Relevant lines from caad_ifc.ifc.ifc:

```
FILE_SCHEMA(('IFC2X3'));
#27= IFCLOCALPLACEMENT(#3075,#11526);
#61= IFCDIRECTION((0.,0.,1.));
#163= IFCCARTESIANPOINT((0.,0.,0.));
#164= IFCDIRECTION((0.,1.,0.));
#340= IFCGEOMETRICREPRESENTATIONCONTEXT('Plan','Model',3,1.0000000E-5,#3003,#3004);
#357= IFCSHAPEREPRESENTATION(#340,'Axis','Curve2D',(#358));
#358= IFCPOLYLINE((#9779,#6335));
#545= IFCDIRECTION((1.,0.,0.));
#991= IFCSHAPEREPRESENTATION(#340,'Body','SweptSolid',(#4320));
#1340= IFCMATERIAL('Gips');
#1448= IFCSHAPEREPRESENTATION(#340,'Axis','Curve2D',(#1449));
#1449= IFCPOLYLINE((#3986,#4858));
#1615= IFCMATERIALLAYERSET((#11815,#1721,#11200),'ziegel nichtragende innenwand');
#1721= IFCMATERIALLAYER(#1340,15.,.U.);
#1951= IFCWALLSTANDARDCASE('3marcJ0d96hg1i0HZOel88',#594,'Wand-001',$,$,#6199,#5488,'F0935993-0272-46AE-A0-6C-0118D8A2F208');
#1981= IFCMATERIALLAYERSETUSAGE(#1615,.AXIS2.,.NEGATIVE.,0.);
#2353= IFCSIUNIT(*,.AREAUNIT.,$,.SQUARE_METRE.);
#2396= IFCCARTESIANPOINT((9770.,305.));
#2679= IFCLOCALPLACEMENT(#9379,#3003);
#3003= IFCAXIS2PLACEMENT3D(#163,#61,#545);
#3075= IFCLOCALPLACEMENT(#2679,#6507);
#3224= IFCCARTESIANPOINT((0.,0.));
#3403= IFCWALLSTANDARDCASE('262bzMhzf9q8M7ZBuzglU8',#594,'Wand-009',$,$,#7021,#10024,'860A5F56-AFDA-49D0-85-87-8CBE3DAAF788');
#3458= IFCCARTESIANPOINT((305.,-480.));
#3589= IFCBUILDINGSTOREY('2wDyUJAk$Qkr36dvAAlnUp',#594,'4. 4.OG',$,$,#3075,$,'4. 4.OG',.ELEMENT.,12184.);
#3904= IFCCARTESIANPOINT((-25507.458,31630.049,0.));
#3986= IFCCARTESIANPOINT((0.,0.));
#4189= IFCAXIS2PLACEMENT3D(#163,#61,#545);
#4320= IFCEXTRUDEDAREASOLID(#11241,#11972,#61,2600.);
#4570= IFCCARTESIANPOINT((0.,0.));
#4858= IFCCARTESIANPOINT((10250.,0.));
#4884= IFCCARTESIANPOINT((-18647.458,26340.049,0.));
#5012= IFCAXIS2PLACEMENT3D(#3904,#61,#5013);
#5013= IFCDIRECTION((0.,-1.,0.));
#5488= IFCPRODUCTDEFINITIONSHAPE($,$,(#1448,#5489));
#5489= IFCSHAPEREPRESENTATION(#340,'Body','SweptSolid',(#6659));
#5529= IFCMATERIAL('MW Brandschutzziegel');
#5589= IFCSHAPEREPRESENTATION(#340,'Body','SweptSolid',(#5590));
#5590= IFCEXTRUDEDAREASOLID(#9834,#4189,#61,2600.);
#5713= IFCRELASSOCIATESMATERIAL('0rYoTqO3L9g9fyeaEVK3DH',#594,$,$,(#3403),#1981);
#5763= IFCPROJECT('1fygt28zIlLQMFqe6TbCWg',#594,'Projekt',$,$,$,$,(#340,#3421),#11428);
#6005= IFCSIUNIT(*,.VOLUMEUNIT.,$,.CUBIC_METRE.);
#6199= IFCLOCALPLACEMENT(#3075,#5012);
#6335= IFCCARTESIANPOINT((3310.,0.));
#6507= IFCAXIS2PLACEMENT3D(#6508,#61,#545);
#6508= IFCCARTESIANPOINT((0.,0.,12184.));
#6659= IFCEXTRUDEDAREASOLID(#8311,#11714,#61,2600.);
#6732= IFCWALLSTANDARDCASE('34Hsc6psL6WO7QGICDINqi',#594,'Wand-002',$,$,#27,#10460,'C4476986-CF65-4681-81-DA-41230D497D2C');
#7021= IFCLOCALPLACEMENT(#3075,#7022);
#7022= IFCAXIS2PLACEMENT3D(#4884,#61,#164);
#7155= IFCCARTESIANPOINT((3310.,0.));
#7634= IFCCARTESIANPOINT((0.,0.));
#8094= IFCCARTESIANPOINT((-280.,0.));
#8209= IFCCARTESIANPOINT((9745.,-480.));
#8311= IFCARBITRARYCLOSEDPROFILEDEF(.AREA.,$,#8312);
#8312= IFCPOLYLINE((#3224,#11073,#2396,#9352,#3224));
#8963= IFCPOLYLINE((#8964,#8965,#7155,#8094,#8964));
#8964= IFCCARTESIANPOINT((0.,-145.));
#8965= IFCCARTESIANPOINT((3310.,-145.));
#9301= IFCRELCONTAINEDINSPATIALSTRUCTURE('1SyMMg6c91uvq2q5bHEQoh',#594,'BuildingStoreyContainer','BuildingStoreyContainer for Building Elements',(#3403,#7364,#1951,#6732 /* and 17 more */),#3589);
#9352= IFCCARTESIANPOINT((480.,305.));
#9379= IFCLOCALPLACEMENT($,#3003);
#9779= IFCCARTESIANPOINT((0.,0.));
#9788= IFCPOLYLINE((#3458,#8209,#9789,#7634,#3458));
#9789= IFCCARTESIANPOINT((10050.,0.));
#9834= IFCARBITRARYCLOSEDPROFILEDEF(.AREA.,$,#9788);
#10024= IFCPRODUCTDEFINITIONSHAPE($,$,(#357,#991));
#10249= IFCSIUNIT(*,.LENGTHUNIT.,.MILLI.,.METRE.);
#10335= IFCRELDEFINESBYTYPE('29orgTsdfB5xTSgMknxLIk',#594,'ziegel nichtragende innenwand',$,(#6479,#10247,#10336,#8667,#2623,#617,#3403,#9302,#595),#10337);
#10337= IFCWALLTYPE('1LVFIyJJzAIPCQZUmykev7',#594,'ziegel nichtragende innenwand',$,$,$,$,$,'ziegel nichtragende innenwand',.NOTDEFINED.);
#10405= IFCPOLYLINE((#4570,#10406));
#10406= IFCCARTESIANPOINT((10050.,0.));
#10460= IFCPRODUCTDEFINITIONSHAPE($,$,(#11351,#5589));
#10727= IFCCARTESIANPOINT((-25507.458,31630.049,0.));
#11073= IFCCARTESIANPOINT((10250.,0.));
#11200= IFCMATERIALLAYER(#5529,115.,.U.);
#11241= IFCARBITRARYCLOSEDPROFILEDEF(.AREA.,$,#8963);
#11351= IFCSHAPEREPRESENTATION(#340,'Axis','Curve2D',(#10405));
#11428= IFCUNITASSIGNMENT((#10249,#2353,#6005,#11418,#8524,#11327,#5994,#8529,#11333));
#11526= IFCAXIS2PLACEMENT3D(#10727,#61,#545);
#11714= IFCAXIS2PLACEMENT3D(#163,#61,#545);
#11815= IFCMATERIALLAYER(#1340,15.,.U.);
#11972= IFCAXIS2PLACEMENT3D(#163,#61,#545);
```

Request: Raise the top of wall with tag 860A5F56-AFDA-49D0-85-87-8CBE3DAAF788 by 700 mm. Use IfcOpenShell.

```python
import ifcopenshell
import ifcopenshell.geom
import ifcopenshell.util.shape
import ifcopenshell.util.unit

model = ifcopenshell.open("caad_ifc.ifc.ifc")
unit_scale = ifcopenshell.util.unit.calculate_unit_scale(model)
settings = ifcopenshell.geom.settings()


def volume(element):
    """Net volume in cubic metres, openings subtracted."""
    shape = ifcopenshell.geom.create_shape(settings, element)
    return ifcopenshell.util.shape.get_volume(shape.geometry)


wall = model.by_guid("262bzMhzf9q8M7ZBuzglU8")
before = volume(wall)

body = next(r for r in wall.Representation.Representations if r.RepresentationIdentifier == "Body")
solid = body.Items[0]
old_height = solid.Depth
solid.Depth += 0.7 / unit_scale
after = volume(wall)

print(f"height {old_height:g} -> {solid.Depth:g}, volume {before:.3f} -> {after:.3f} m3")

model.write("caad_ifc.ifc_rev.ifc")
```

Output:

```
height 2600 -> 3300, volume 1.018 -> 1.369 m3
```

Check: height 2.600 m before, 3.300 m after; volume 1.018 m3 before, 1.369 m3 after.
